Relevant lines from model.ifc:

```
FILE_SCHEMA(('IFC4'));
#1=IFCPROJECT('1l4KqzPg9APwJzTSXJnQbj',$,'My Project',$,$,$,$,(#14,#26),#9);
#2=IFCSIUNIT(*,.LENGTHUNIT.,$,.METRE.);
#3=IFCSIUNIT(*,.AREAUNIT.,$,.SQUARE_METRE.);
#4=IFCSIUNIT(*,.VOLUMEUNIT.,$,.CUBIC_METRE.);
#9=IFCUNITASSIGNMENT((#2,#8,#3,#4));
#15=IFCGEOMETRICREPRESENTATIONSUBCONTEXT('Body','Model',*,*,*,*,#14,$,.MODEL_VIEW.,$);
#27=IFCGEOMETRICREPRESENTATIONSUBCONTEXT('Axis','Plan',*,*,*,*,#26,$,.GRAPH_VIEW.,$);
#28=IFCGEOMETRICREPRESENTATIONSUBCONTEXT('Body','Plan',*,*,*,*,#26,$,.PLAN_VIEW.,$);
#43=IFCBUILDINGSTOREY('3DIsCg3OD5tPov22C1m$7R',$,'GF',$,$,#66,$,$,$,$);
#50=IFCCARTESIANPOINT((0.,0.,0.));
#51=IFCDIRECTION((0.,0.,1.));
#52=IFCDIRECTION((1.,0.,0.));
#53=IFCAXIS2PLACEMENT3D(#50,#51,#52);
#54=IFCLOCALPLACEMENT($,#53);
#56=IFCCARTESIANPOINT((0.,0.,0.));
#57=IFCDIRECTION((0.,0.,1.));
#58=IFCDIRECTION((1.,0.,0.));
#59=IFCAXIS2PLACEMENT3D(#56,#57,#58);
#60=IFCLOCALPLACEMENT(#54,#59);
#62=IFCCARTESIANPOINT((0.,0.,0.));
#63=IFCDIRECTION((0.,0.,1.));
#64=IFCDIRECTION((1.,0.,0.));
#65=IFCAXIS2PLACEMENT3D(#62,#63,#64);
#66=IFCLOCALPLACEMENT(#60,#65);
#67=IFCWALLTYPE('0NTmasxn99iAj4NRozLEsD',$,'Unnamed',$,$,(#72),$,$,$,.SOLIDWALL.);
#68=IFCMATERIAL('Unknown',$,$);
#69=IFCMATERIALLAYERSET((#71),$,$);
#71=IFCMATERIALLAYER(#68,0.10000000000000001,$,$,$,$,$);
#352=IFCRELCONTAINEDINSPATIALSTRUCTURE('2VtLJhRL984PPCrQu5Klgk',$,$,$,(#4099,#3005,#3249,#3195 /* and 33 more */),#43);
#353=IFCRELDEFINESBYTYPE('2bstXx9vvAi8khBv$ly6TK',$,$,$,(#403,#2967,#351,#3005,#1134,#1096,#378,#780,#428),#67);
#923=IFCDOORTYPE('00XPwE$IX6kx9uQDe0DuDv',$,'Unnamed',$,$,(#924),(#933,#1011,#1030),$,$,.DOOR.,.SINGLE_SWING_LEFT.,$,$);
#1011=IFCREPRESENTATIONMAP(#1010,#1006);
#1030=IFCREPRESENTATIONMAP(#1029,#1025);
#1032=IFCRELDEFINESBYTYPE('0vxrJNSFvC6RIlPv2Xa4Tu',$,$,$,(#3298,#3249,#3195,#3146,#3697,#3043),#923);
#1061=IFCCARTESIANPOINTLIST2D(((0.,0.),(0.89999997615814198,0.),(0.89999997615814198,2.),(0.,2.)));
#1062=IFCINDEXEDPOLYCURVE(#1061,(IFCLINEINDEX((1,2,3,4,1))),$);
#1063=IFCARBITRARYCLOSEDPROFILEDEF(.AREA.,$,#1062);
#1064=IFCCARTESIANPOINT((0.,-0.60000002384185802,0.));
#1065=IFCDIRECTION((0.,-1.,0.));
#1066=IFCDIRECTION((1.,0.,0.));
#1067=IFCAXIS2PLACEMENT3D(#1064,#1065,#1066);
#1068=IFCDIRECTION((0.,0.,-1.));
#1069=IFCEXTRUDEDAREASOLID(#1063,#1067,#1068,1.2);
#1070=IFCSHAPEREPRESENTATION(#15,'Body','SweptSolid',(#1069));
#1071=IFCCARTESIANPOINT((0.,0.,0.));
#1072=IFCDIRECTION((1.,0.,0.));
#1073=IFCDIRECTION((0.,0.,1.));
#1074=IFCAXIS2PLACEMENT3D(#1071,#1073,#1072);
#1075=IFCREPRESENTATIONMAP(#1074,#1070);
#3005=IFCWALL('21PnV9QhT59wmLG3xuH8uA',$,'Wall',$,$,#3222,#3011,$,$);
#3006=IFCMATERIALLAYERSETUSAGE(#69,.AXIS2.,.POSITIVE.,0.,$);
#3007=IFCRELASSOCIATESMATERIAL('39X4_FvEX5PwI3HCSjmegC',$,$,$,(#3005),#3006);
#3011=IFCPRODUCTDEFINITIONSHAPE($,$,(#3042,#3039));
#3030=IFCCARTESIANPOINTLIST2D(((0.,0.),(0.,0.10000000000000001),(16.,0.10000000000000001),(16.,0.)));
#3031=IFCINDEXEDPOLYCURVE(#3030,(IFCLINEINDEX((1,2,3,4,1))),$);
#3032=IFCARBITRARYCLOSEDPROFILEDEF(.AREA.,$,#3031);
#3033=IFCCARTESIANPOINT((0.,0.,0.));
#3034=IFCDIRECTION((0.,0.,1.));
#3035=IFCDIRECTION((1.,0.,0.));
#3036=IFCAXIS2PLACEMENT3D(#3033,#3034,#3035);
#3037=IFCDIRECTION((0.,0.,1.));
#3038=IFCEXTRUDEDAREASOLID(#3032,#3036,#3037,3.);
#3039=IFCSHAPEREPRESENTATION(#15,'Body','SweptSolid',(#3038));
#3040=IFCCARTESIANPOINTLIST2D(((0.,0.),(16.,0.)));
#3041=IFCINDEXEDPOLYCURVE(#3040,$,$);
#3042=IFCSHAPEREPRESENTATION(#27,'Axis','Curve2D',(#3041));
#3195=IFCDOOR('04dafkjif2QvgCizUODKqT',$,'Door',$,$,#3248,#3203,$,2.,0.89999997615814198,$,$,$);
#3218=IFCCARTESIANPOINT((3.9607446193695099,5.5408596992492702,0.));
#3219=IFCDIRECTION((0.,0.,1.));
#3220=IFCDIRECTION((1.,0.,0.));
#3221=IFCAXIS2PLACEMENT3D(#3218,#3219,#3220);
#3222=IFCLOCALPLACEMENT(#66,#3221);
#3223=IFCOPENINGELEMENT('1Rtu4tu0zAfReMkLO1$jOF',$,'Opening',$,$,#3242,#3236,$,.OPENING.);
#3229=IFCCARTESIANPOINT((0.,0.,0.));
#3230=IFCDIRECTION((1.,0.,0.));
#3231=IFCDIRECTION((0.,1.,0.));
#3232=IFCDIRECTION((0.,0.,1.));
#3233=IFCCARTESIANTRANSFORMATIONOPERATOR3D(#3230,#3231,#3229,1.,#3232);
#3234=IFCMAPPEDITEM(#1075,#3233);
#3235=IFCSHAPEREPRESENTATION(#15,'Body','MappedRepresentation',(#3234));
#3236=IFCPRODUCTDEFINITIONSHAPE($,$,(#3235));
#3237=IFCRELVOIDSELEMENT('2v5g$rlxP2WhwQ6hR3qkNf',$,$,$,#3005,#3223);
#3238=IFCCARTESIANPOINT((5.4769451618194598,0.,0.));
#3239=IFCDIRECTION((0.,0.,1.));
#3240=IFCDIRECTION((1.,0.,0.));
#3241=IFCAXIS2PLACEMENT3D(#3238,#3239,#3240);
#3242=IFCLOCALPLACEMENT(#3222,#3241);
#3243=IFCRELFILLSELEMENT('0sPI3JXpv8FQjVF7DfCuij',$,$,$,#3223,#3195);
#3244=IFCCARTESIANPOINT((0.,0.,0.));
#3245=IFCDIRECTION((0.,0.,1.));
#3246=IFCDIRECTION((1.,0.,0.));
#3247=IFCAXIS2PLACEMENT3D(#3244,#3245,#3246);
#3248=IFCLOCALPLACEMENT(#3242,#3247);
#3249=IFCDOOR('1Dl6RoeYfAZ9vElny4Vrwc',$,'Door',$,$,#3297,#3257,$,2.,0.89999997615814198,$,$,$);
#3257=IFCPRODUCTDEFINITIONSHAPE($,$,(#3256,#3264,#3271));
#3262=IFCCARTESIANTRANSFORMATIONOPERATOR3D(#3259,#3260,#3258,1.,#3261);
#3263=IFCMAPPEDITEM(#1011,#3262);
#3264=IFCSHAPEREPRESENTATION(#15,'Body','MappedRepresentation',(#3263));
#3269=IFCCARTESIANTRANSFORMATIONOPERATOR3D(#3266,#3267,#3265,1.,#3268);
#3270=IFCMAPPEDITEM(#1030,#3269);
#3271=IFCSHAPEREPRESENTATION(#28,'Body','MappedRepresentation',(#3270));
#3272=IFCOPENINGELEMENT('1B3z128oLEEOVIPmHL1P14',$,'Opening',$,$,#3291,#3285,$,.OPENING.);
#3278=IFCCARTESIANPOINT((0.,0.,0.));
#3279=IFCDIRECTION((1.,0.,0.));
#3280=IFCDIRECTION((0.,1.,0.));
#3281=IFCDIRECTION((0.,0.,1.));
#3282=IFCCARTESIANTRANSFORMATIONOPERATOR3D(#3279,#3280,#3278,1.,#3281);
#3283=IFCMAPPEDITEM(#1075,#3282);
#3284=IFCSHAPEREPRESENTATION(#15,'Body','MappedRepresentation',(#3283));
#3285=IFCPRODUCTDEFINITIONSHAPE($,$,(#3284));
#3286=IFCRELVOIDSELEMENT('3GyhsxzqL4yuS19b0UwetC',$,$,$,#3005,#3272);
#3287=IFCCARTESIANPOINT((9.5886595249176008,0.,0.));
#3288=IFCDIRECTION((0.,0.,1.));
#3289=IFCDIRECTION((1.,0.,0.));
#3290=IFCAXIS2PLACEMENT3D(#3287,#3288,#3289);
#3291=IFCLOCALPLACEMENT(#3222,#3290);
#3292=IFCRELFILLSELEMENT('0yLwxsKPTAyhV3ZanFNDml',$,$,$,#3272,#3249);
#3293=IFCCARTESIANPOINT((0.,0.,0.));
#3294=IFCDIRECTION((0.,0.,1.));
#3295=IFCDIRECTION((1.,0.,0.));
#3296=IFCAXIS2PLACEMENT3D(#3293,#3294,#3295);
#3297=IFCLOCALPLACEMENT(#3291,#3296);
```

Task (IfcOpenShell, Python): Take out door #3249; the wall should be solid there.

```python
import ifcopenshell
import ifcopenshell.api.feature
import ifcopenshell.api.root
import ifcopenshell.geom
import ifcopenshell.util.shape

model = ifcopenshell.open("model.ifc")
settings = ifcopenshell.geom.settings()


def volume(element):
    """Net volume in cubic metres, openings subtracted."""
    shape = ifcopenshell.geom.create_shape(settings, element)
    return ifcopenshell.util.shape.get_volume(shape.geometry)


door = model.by_guid("1Dl6RoeYfAZ9vElny4Vrwc")
opening = door.FillsVoids[0].RelatingOpeningElement
wall = opening.VoidsElements[0].RelatingBuildingElement
before = volume(wall)

ifcopenshell.api.root.remove_product(model, product=door)
ifcopenshell.api.feature.remove_feature(model, feature=opening)

after = volume(wall)

print(f"wall volume {before:.3f} -> {after:.3f} m3")

model.write("model_edited.ifc")
```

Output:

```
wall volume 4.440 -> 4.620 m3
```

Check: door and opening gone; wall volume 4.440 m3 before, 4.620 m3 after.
